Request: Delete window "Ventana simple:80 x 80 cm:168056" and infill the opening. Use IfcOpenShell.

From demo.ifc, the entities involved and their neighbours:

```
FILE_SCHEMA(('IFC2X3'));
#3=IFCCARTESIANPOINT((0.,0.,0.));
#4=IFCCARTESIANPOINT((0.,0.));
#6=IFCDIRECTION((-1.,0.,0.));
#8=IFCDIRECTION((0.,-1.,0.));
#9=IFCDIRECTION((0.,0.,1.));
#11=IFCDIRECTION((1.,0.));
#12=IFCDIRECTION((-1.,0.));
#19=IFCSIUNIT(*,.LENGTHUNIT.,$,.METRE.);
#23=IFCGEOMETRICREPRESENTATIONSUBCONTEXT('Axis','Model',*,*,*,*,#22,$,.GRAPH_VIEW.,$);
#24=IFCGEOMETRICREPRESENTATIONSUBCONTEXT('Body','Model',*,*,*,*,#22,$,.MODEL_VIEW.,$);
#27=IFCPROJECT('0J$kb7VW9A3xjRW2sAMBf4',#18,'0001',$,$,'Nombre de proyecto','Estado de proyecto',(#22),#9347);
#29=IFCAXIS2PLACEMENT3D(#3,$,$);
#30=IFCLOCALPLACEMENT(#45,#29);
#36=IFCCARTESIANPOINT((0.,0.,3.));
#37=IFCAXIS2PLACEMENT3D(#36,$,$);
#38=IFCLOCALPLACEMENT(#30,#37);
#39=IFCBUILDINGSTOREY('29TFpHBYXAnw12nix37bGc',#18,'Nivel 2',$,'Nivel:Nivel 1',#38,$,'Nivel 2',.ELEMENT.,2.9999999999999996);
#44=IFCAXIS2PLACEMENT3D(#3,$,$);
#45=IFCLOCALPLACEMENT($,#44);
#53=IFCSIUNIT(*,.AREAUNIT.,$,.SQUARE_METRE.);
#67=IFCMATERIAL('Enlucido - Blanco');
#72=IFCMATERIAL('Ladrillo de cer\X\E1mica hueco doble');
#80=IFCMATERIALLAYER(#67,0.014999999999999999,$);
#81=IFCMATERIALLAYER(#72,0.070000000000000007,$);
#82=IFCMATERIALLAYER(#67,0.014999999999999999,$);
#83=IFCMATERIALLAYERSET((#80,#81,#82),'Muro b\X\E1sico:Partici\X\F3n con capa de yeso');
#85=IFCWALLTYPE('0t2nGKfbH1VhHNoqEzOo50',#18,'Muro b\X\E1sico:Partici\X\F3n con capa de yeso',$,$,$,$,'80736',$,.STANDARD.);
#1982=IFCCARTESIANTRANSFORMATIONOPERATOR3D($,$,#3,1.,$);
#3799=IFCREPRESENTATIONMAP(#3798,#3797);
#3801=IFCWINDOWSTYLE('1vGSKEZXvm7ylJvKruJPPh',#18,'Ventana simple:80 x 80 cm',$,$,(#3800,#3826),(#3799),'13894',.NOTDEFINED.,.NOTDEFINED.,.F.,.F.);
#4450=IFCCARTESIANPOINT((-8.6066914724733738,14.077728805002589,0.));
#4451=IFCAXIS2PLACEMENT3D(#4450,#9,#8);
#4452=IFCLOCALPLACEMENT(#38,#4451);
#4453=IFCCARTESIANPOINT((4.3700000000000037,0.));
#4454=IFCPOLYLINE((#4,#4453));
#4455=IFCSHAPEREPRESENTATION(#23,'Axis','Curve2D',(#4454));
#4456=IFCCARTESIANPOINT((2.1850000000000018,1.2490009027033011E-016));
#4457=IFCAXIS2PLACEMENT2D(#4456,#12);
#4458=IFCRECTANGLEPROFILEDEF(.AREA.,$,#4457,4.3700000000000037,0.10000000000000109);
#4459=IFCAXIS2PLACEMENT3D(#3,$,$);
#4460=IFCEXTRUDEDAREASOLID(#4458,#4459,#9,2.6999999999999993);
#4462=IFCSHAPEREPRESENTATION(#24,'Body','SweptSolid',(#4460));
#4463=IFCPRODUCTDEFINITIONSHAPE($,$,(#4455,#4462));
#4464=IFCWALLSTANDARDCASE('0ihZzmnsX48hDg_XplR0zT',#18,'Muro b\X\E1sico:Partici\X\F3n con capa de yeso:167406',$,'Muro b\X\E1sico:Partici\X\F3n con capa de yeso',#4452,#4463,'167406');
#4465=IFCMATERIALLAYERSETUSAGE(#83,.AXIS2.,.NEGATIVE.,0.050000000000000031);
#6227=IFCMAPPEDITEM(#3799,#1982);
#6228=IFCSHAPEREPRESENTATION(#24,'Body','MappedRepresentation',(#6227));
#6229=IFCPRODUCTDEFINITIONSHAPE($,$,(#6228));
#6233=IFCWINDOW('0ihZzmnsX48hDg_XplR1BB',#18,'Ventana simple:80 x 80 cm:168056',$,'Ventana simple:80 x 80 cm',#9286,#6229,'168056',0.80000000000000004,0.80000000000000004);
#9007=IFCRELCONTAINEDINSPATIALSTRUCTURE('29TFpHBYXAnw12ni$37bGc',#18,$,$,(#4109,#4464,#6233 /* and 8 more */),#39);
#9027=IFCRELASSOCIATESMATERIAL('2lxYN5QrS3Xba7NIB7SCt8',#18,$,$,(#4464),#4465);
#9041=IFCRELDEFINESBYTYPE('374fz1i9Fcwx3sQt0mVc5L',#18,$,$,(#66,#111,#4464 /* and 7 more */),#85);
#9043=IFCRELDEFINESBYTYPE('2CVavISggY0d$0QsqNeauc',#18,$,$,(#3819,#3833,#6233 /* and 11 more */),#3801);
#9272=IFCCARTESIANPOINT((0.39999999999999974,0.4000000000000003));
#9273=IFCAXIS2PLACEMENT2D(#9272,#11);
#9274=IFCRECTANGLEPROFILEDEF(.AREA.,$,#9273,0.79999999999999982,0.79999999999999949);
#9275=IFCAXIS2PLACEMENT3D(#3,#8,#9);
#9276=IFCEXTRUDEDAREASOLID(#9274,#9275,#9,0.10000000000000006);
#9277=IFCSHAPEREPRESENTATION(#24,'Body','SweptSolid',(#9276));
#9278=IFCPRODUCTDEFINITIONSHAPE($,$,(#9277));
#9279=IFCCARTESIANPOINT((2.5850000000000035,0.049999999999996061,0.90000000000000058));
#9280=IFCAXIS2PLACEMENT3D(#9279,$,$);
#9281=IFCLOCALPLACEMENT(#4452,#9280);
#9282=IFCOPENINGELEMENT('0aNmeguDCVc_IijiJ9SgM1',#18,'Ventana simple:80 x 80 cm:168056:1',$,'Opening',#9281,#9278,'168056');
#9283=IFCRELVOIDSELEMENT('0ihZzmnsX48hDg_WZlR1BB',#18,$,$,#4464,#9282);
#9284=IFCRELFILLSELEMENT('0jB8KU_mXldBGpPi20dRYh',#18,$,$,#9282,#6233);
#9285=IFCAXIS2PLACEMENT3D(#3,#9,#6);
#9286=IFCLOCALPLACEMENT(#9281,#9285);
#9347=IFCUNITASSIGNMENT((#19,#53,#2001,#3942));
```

```python
import ifcopenshell
import ifcopenshell.api.feature
import ifcopenshell.api.root
import ifcopenshell.geom
import ifcopenshell.util.shape

model = ifcopenshell.open("demo.ifc")
settings = ifcopenshell.geom.settings()


def volume(element):
    """Net volume in cubic metres, openings subtracted."""
    shape = ifcopenshell.geom.create_shape(settings, element)
    return ifcopenshell.util.shape.get_volume(shape.geometry)


window = model.by_guid("0ihZzmnsX48hDg_XplR1BB")
opening = window.FillsVoids[0].RelatingOpeningElement
wall = opening.VoidsElements[0].RelatingBuildingElement
before = volume(wall)

ifcopenshell.api.root.remove_product(model, product=window)
ifcopenshell.api.feature.remove_feature(model, feature=opening)

after = volume(wall)

print(f"wall volume {before:.3f} -> {after:.3f} m3")

model.write("demo_updated.ifc")
```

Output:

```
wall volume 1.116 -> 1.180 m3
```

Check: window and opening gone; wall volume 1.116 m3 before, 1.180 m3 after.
